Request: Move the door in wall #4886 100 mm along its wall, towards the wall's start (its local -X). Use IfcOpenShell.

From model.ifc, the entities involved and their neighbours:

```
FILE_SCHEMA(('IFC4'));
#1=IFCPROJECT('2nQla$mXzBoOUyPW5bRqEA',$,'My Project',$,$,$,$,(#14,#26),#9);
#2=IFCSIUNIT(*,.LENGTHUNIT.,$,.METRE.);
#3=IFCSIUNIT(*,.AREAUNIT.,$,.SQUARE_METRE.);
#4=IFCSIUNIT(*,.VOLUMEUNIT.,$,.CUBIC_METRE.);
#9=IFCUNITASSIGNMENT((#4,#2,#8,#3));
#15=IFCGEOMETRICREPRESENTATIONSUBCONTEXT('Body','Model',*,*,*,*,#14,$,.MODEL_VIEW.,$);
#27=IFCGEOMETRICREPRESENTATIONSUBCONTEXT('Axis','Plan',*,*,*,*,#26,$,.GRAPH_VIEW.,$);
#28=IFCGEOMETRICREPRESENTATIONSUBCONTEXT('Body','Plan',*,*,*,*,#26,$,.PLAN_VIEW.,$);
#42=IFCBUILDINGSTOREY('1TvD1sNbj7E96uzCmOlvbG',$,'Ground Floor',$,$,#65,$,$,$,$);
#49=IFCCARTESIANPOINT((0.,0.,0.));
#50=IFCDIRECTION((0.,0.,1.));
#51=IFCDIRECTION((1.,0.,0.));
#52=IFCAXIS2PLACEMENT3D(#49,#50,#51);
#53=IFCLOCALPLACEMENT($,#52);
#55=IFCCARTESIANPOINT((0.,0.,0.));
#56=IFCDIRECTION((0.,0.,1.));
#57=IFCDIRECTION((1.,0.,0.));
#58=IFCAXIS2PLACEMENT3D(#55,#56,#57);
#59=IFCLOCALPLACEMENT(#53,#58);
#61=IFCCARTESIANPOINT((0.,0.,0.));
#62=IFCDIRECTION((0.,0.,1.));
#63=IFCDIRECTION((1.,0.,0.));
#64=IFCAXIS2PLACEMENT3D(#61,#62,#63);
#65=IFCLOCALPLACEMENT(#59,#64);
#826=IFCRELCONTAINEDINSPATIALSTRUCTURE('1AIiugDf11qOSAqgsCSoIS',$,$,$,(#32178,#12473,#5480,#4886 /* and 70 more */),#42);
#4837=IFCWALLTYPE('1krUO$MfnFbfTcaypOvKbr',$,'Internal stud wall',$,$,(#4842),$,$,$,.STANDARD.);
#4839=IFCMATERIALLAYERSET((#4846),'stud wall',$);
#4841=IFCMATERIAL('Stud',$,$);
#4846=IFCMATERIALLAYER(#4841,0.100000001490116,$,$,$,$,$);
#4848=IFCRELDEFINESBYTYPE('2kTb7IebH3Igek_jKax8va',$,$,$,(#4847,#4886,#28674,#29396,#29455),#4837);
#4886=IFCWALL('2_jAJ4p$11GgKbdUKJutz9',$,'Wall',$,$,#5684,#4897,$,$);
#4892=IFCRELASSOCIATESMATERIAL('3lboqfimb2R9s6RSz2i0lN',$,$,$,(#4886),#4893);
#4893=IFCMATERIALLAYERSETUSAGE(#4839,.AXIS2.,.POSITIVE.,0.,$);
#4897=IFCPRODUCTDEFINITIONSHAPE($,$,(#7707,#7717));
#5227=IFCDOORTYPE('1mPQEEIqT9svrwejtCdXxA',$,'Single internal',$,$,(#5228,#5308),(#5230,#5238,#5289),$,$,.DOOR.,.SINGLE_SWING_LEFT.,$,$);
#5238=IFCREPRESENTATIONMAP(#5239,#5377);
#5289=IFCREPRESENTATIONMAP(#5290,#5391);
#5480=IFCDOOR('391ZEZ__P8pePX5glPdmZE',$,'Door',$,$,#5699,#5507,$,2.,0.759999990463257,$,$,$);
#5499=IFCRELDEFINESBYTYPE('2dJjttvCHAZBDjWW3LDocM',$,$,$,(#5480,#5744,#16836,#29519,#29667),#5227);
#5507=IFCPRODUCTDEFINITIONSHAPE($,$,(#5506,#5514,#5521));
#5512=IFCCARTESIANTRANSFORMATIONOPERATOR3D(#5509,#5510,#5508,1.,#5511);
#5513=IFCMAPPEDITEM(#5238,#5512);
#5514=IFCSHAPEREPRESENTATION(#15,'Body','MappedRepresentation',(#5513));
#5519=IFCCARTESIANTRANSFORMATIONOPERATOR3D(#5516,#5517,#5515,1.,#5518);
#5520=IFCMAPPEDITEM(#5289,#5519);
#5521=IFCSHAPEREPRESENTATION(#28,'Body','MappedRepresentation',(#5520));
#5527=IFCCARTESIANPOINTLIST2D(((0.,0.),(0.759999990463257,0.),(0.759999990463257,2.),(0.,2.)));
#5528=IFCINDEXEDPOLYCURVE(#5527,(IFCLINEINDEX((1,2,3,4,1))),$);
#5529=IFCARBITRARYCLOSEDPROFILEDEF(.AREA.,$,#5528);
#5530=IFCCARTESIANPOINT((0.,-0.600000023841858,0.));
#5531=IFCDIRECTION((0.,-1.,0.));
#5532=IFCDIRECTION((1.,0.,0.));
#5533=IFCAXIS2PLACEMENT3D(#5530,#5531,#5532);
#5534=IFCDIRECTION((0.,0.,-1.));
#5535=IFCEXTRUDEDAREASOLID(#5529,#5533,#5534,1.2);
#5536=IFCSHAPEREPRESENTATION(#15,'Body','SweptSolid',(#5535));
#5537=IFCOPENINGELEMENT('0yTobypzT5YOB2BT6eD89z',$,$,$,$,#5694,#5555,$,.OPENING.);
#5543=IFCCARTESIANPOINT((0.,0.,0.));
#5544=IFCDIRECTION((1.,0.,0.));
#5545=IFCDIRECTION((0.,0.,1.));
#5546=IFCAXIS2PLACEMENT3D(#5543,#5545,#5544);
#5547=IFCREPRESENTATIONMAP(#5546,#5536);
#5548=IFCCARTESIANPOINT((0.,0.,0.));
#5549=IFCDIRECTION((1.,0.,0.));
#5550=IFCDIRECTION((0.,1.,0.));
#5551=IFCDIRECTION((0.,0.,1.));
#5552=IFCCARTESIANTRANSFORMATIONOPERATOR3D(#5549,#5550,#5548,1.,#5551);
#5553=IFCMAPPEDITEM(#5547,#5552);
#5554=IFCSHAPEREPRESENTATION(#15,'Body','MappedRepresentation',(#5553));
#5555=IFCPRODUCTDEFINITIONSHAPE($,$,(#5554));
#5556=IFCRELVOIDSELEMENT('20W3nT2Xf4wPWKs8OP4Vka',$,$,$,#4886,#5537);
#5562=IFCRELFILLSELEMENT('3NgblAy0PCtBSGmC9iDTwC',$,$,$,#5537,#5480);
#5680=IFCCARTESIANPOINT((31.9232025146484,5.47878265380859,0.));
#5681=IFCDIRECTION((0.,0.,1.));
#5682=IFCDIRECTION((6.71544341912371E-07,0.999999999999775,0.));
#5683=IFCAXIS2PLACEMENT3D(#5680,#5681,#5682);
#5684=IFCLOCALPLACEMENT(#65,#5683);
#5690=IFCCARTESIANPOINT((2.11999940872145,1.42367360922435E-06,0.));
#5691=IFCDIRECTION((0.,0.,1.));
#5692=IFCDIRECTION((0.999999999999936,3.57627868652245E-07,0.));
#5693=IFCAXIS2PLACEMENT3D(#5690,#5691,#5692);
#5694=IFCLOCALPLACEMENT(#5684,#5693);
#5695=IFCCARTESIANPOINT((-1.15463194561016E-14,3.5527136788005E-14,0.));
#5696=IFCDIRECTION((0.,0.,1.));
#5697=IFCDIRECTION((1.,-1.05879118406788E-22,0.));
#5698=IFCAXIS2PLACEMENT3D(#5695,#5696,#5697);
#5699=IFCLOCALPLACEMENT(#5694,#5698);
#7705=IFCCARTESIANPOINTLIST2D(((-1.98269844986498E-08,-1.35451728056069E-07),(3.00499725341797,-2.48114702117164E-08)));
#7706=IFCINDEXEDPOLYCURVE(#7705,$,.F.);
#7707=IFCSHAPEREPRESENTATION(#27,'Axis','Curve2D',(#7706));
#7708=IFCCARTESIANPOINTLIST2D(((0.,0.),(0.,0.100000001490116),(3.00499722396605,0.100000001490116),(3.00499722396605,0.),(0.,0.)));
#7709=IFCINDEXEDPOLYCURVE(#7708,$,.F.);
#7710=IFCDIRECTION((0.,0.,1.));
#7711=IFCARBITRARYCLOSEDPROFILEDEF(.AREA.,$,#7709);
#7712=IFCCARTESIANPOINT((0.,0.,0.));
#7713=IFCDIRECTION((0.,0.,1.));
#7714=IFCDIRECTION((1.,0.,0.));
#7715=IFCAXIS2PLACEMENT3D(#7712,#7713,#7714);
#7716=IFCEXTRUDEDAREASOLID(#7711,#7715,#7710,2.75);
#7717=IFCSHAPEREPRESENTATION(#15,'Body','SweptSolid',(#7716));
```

```python
import ifcopenshell
import ifcopenshell.api.geometry
import ifcopenshell.util.placement
import ifcopenshell.util.unit

model = ifcopenshell.open("model.ifc")
unit_scale = ifcopenshell.util.unit.calculate_unit_scale(model)

door = model.by_guid("391ZEZ__P8pePX5glPdmZE")
opening = door.FillsVoids[0].RelatingOpeningElement
wall = opening.VoidsElements[0].RelatingBuildingElement

wall_matrix = ifcopenshell.util.placement.get_local_placement(wall.ObjectPlacement)
shift = wall_matrix[:3, 0] * -0.1 / unit_scale
before = ifcopenshell.util.placement.get_local_placement(door.ObjectPlacement)[:3, 3].copy()

# The door is placed relative to its opening, so it follows when the opening moves.
matrix = ifcopenshell.util.placement.get_local_placement(opening.ObjectPlacement)
matrix[:3, 3] += shift
ifcopenshell.api.geometry.edit_object_placement(
    model, product=opening, matrix=matrix, is_si=False, should_transform_children=True
)

after = ifcopenshell.util.placement.get_local_placement(door.ObjectPlacement)[:3, 3]
print("door moved by", (after - before).round(3) + 0.0)

model.write("model_rev.ifc")
```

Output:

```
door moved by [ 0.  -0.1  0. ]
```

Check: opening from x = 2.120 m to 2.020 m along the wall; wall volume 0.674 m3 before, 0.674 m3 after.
